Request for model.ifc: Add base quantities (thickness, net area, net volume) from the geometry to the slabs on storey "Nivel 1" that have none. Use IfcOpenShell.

First a look at what the model holds.

```python
import ifcopenshell
import ifcopenshell.util.element
import ifcopenshell.util.unit

model = ifcopenshell.open("model.ifc")
print(model.schema)
for unit_type in ("LENGTHUNIT", "AREAUNIT", "VOLUMEUNIT"):
    print(unit_type, ifcopenshell.util.unit.calculate_unit_scale(model, unit_type))
storey = next(s for s in model.by_type("IfcBuildingStorey") if s.Name == "Nivel 1")
slabs = [e for e in ifcopenshell.util.element.get_decomposition(storey) if e.is_a("IfcSlab")]
for e in sorted(slabs, key=lambda e: e.id()):
    print(e.id(), e.is_a(), e.Name, list(ifcopenshell.util.element.get_psets(e, qtos_only=True)), sep=" | ")
```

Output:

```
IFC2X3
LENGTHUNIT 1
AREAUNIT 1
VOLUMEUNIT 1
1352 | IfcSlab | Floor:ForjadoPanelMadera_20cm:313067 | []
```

```python
import ifcopenshell
import ifcopenshell.api.pset
import ifcopenshell.geom
import ifcopenshell.util.element
import ifcopenshell.util.shape
import ifcopenshell.util.unit

model = ifcopenshell.open("model.ifc")
unit_scale = ifcopenshell.util.unit.calculate_unit_scale(model)
area_scale = ifcopenshell.util.unit.calculate_unit_scale(model, "AREAUNIT")
volume_scale = ifcopenshell.util.unit.calculate_unit_scale(model, "VOLUMEUNIT")
settings = ifcopenshell.geom.settings()

storey = next(s for s in model.by_type("IfcBuildingStorey") if s.Name == "Nivel 1")
slabs = [e for e in ifcopenshell.util.element.get_decomposition(storey) if e.is_a("IfcSlab")]

for e in sorted(slabs, key=lambda e: e.id()):
    if ifcopenshell.util.element.get_psets(e, qtos_only=True, should_inherit=False):
        continue
    # Geometry comes back in metres, in the element's own axes.
    shape = ifcopenshell.geom.create_shape(settings, e)
    values = {
        "Width": ifcopenshell.util.shape.get_z(shape.geometry) / unit_scale,
        "NetArea": ifcopenshell.util.shape.get_footprint_area(shape.geometry) / area_scale,
        "NetVolume": ifcopenshell.util.shape.get_volume(shape.geometry) / volume_scale,
    }
    qto = ifcopenshell.api.pset.add_qto(model, product=e, name="BaseQuantities")
    ifcopenshell.api.pset.edit_qto(model, qto=qto, properties=values)
    print(e.id(), {k: round(v, 3) for k, v in values.items()})

model.write("model_updated.ifc")
```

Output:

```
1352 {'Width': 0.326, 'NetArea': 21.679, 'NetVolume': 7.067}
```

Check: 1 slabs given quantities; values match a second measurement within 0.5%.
